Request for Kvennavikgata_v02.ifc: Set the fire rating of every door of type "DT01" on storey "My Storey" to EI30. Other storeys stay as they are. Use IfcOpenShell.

First a look at what the model holds.

```python
import ifcopenshell
import ifcopenshell.util.element

model = ifcopenshell.open("Kvennavikgata_v02.ifc")
print(model.schema)
storey = next(s for s in model.by_type("IfcBuildingStorey") if s.Name == "My Storey")
doors = [e for e in ifcopenshell.util.element.get_decomposition(storey) if e.is_a("IfcDoor")]
seen = {}
for e in doors:
    element_type = ifcopenshell.util.element.get_type(e)
    key = (element_type.Name if element_type != e and element_type else None, ifcopenshell.util.element.get_pset(e, "Pset_DoorCommon", "FireRating"))
    seen[key] = seen.get(key, 0) + 1
for (name, value), count in sorted(seen.items(), key=str):
    print(count, "x", name, "|", value)
```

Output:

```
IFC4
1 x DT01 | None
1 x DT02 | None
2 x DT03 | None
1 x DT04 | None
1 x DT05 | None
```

```python
import ifcopenshell
import ifcopenshell.api.pset
import ifcopenshell.util.element

model = ifcopenshell.open("Kvennavikgata_v02.ifc")

storey = next(s for s in model.by_type("IfcBuildingStorey") if s.Name == "My Storey")
doors = [e for e in ifcopenshell.util.element.get_decomposition(storey) if e.is_a("IfcDoor")]

count = 0
for e in doors:
    element_type = ifcopenshell.util.element.get_type(e)
    if element_type in (None, e) or element_type.Name != "DT01":
        continue
    # add_pset returns the element's existing set when there is one.
    pset = ifcopenshell.api.pset.add_pset(model, product=e, name="Pset_DoorCommon")
    ifcopenshell.api.pset.edit_pset(model, pset=pset, properties={"FireRating": "EI30"})
    count += 1

print(count, "doors updated")

model.write("Kvennavikgata_v02-out.ifc")
```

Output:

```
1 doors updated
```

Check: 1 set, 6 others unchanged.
